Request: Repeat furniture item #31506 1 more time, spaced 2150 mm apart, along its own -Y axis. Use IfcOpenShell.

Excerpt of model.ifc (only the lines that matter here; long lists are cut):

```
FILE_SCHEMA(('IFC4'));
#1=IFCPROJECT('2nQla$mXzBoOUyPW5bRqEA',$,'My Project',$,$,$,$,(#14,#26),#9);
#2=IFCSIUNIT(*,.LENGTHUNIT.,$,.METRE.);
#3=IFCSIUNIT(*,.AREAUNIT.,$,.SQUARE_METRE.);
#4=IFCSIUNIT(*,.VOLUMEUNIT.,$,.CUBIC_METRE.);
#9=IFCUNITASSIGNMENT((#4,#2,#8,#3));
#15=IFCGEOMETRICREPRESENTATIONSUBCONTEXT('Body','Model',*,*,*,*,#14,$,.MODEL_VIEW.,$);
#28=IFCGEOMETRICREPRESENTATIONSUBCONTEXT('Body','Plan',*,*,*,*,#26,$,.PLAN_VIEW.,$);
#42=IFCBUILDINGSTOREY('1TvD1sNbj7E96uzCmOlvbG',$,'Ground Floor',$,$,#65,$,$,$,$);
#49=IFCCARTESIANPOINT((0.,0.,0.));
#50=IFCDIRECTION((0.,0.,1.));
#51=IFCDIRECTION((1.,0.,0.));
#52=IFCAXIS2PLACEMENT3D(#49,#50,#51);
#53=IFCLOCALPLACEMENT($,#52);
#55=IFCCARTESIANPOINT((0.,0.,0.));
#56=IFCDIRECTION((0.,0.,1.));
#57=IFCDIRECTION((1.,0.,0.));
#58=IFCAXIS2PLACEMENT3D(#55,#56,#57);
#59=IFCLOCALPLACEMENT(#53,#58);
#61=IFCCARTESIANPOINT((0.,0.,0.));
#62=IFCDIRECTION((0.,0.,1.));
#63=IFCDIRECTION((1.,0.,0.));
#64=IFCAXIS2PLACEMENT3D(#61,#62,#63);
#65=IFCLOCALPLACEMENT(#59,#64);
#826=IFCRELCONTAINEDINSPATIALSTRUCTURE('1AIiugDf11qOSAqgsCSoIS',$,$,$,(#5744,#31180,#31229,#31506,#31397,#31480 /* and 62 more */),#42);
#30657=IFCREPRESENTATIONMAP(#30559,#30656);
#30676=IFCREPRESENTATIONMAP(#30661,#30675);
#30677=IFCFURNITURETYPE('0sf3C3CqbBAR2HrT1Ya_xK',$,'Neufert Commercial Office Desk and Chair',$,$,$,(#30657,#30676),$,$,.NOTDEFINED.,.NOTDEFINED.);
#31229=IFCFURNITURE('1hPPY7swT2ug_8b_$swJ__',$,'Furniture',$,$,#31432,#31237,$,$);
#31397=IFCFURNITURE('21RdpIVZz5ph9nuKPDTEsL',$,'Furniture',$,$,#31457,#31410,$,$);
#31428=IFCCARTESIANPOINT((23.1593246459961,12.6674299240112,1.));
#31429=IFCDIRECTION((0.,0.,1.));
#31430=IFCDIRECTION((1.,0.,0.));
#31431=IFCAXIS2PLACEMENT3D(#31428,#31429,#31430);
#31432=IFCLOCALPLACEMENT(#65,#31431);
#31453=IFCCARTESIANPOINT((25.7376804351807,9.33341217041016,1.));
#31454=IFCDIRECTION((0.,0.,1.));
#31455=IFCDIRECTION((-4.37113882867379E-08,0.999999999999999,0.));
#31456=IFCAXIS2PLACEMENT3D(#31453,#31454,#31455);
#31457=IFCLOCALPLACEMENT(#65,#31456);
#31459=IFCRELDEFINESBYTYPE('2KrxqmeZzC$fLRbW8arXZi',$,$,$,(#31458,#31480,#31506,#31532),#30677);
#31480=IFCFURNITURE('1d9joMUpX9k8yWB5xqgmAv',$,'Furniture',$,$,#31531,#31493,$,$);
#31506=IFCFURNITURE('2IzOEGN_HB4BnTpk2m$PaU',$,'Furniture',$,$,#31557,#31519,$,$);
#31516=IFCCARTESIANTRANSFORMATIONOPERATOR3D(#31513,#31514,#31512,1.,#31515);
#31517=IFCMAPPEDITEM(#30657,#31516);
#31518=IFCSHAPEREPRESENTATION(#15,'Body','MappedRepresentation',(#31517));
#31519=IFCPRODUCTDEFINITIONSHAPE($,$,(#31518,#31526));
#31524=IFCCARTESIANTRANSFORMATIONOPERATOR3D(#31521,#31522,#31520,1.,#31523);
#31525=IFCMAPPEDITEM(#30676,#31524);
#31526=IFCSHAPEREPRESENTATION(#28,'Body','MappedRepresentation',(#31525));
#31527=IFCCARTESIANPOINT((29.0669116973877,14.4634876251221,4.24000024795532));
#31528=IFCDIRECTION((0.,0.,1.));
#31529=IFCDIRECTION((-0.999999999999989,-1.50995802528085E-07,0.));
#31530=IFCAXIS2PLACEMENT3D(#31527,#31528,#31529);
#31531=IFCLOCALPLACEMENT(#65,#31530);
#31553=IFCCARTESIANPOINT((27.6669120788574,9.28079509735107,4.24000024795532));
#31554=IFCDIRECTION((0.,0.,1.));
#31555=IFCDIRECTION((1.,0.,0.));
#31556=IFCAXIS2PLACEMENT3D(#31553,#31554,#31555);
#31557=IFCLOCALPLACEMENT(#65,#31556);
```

```python
import ifcopenshell
import ifcopenshell.api.geometry
import ifcopenshell.api.root
import ifcopenshell.util.element
import ifcopenshell.util.placement

model = ifcopenshell.open("model.ifc")

source = model.by_guid("2IzOEGN_HB4BnTpk2m$PaU")
base = ifcopenshell.util.placement.get_local_placement(source.ObjectPlacement)
step = -base[:3, 1] * 2.15

for i in range(1, 2):
    copy = ifcopenshell.api.root.copy_class(model, product=source)
    copy.Representation = ifcopenshell.util.element.copy_deep(
        model, source.Representation, exclude=["IfcGeometricRepresentationContext", "IfcRepresentationMap"]
    )
    matrix = base.copy()
    matrix[:3, 3] += i * step
    print("added at", matrix[:3, 3].round(3) + 0.0)
    ifcopenshell.api.geometry.edit_object_placement(model, product=copy, matrix=matrix, is_si=False)

model.write("model_v2.ifc")
```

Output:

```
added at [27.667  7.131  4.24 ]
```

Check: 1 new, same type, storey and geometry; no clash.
